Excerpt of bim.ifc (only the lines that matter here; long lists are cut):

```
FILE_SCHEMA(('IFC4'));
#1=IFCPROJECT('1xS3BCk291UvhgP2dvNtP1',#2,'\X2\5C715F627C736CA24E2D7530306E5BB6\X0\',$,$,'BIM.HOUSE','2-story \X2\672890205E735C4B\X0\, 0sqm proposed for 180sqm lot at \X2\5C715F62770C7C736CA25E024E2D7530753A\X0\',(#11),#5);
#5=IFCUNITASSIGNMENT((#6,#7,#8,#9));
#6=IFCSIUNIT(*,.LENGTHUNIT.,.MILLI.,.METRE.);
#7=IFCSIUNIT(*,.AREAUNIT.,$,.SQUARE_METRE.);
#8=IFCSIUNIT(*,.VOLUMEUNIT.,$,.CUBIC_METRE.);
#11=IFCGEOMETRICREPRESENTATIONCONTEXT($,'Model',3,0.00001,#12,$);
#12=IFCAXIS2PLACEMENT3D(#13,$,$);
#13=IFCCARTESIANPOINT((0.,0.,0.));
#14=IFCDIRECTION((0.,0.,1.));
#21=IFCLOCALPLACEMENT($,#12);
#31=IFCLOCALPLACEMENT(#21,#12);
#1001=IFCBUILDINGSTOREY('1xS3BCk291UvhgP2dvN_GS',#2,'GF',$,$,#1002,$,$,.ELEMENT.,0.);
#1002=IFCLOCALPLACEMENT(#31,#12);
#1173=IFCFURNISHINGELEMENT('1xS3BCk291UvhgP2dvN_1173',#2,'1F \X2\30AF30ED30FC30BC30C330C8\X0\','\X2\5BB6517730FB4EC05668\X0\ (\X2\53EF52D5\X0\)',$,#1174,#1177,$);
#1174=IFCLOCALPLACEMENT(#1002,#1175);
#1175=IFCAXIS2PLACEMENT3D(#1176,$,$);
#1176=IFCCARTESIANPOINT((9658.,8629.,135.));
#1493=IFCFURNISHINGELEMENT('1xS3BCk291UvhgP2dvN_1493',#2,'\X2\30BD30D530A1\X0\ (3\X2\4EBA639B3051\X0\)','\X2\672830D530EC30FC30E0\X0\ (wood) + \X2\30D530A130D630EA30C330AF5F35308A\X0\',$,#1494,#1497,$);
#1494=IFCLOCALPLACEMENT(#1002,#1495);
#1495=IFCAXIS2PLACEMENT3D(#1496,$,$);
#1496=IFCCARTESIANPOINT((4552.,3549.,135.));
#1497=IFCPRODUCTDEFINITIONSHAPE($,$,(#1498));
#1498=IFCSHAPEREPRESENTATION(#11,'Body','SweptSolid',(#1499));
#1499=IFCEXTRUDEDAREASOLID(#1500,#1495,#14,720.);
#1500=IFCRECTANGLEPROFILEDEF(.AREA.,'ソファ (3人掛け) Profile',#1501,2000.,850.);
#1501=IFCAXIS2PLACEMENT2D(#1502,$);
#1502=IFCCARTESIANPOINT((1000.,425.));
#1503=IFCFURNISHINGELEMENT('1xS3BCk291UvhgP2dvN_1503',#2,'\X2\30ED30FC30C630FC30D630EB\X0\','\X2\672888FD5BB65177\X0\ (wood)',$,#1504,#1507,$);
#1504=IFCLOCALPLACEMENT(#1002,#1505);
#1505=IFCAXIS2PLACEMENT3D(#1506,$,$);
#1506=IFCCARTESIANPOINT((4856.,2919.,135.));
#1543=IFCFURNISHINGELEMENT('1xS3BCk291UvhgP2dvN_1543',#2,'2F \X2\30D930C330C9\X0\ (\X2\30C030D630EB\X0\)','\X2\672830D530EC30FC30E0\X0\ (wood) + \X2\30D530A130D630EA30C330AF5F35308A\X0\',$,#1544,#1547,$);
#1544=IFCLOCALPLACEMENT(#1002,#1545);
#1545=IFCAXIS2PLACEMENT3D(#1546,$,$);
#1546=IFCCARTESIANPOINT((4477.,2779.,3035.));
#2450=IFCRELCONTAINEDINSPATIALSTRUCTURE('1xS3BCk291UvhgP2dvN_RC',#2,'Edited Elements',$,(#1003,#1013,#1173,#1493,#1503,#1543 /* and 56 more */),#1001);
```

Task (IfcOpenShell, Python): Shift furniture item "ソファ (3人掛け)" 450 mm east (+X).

```python
import ifcopenshell
import ifcopenshell.api.geometry
import ifcopenshell.util.placement

model = ifcopenshell.open("bim.ifc")

item = model.by_guid("1xS3BCk291UvhgP2dvN_1493")
matrix = ifcopenshell.util.placement.get_local_placement(item.ObjectPlacement)
matrix[0, 3] += 450.0
ifcopenshell.api.geometry.edit_object_placement(model, product=item, matrix=matrix, is_si=False)

print(ifcopenshell.util.placement.get_local_placement(item.ObjectPlacement).round(3) + 0.0)

model.write("bim_updated.ifc")
```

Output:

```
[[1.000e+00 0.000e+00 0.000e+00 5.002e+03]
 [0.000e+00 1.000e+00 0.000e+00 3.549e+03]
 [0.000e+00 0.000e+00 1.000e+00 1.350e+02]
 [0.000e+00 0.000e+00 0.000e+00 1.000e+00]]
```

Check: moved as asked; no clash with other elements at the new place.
